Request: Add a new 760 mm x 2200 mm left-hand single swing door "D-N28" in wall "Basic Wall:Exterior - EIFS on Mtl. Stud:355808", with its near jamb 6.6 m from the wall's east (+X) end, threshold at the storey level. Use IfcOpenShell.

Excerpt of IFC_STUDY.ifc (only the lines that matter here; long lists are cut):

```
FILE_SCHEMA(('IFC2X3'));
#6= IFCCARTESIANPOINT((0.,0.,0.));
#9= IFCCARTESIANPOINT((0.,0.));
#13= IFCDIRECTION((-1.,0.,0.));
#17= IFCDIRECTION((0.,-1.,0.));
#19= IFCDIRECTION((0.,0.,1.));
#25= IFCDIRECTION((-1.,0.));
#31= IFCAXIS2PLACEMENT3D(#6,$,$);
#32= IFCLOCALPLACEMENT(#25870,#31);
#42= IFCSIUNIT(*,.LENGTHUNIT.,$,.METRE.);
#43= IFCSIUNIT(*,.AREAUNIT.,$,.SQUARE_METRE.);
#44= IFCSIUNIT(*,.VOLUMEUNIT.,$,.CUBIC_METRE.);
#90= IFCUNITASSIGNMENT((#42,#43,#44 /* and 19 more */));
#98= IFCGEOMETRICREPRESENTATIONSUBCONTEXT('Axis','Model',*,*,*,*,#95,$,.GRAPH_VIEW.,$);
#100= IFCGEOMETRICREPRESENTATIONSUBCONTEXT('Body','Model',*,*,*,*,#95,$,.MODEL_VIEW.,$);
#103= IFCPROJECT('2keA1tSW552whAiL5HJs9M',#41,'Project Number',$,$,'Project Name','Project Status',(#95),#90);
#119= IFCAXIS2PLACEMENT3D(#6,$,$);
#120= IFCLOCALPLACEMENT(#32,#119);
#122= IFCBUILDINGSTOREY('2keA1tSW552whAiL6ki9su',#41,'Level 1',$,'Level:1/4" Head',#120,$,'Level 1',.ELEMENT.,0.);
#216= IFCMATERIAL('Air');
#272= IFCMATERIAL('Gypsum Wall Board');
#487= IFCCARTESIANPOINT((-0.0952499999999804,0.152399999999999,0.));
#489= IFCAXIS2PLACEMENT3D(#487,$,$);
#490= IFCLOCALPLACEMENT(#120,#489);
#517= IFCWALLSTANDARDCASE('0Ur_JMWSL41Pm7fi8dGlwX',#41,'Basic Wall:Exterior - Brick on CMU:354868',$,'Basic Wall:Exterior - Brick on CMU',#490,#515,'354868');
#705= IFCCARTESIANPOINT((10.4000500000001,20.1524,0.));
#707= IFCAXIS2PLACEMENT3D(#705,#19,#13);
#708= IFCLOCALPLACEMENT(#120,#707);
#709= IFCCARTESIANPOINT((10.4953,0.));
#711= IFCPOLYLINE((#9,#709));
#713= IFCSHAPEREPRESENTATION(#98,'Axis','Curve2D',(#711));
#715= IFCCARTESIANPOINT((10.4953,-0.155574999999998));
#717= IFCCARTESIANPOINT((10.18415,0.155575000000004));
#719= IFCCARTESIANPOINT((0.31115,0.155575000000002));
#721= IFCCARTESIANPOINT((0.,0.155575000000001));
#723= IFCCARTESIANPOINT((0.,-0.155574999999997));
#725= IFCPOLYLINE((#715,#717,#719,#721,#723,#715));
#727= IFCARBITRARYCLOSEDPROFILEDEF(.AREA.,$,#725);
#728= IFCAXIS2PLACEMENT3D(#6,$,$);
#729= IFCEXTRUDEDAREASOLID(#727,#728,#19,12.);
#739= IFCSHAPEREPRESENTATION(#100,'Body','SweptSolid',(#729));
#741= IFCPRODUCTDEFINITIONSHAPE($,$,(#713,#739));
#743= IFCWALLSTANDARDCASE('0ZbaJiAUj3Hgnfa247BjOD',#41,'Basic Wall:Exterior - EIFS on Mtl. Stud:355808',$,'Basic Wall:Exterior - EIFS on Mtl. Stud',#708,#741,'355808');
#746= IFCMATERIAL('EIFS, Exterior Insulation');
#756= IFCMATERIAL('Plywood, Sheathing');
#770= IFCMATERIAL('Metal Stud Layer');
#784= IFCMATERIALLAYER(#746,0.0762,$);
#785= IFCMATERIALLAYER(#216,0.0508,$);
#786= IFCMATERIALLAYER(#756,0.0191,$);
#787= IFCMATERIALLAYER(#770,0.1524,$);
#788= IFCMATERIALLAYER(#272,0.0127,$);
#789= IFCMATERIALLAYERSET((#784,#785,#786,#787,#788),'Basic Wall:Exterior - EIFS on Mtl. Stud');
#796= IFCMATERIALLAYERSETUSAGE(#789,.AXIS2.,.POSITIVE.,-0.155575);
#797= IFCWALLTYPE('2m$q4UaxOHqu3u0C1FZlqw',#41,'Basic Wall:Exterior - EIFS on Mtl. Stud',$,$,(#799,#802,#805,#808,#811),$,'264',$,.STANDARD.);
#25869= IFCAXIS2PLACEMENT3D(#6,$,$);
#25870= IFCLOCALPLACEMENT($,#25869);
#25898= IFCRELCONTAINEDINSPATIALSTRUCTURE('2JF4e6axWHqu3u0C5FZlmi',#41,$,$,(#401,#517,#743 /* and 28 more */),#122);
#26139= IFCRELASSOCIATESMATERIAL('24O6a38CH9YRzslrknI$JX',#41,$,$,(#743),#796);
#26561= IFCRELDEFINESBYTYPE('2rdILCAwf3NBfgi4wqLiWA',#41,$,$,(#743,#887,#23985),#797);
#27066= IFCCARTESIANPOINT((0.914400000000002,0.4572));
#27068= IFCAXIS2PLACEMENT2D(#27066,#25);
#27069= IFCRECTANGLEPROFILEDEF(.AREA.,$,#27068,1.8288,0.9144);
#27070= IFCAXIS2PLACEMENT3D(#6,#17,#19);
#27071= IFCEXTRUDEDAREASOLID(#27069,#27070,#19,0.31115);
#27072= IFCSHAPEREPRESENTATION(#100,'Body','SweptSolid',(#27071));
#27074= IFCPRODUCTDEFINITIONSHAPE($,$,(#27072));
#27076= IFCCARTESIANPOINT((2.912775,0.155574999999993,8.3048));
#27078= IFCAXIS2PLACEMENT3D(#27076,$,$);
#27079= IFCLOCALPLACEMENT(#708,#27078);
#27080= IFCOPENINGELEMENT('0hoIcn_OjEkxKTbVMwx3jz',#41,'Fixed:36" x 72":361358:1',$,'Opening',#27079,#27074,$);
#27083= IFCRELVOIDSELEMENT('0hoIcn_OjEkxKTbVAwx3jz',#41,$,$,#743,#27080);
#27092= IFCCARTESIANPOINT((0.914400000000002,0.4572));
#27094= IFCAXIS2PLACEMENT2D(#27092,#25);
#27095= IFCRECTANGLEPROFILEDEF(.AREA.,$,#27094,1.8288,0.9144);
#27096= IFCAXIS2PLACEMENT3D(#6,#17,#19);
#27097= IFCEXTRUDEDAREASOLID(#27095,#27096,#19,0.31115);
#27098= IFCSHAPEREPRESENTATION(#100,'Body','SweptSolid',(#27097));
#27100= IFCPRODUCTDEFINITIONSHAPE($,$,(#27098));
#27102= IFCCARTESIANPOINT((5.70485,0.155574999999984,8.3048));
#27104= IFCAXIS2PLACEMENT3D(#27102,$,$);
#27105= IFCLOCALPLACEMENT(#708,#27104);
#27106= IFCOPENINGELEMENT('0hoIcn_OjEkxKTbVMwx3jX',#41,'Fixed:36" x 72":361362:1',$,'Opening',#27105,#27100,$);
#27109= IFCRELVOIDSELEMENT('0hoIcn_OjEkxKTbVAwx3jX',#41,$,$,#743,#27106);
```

```python
import numpy as np
import ifcopenshell
import ifcopenshell.api.feature
import ifcopenshell.api.geometry
import ifcopenshell.api.root
import ifcopenshell.api.spatial
import ifcopenshell.api.type
import ifcopenshell.geom
import ifcopenshell.util.element
import ifcopenshell.util.placement
import ifcopenshell.util.representation
import ifcopenshell.util.shape
import ifcopenshell.util.unit

model = ifcopenshell.open("IFC_STUDY.ifc")
unit_scale = ifcopenshell.util.unit.calculate_unit_scale(model)
settings = ifcopenshell.geom.settings()


def volume(element):
    """Net volume in cubic metres, openings subtracted."""
    shape = ifcopenshell.geom.create_shape(settings, element)
    return ifcopenshell.util.shape.get_volume(shape.geometry)


wall = model.by_id(743)
storey = ifcopenshell.util.element.get_container(wall, ifc_class="IfcBuildingStorey")
context = ifcopenshell.util.representation.get_context(model, "Model", "Body", "MODEL_VIEW")
before = volume(wall)

width, height, from_end, sill = 0.76, 2.2, 6.6, 0.0  # metres

# The wall runs along its own X axis, and the end named is its -X end.
wall_shape = ifcopenshell.geom.create_shape(settings, wall)
x, y, z = ifcopenshell.util.shape.get_vertices(wall_shape.geometry).T
start = x.min() + from_end
face, thickness = float(y.min()), float(y.max() - y.min())
wall_matrix = ifcopenshell.util.placement.get_local_placement(wall.ObjectPlacement)
level = ifcopenshell.util.placement.get_local_placement(storey.ObjectPlacement)[2, 3]


def in_wall(x, y):
    """Placement at x, y metres in the wall's axes, at sill height."""
    matrix = wall_matrix.copy()
    matrix[:, 3] = wall_matrix @ np.array([x / unit_scale, y / unit_scale, 0.0, 1.0])
    matrix[2, 3] = level + sill / unit_scale
    return matrix


# Opening: a box that overshoots both wall faces by 50 mm.
opening = ifcopenshell.api.root.create_entity(model, ifc_class="IfcOpeningElement")
box = ifcopenshell.api.geometry.add_wall_representation(
    model, context=context, length=width, height=height, thickness=thickness + 0.1
)
ifcopenshell.api.geometry.assign_representation(model, product=opening, representation=box)
ifcopenshell.api.geometry.edit_object_placement(model, product=opening, matrix=in_wall(start, face - 0.05), is_si=False)
ifcopenshell.api.feature.add_feature(model, feature=opening, element=wall)

door = ifcopenshell.api.root.create_entity(model, ifc_class="IfcDoor", name="D-N28")
door.OverallWidth, door.OverallHeight = width / unit_scale, height / unit_scale
body = ifcopenshell.api.geometry.add_door_representation(
    model,
    context=context,
    overall_width=door.OverallWidth,
    overall_height=door.OverallHeight,
    operation_type="SINGLE_SWING_LEFT",
    lining_properties={"LiningDepth": thickness / unit_scale, "ThresholdDepth": thickness / unit_scale},
)
ifcopenshell.api.geometry.assign_representation(model, product=door, representation=body)
ifcopenshell.api.spatial.assign_container(model, products=[door], relating_structure=storey)
fills = ifcopenshell.api.feature.add_filling(model, opening=opening, element=door)
fills.OwnerHistory = door.OwnerHistory  # required in IFC2X3

# IFC2X3 keeps the operation on the door style.
style = ifcopenshell.api.root.create_entity(model, ifc_class="IfcDoorStyle", name="D-N28")
style.OperationType, style.ConstructionType = "SINGLE_SWING_LEFT", "NOTDEFINED"
style.ParameterTakesPrecedence = style.Sizeable = False
ifcopenshell.api.type.assign_type(model, related_objects=[door], relating_type=style)

# The lining spans the wall, so the door starts at the wall face.
ifcopenshell.api.geometry.edit_object_placement(model, product=door, matrix=in_wall(start, face), is_si=False)

after = volume(wall)

print(f"wall volume {before:.3f} -> {after:.3f} m3")

model.write("IFC_STUDY_updated.ifc")
```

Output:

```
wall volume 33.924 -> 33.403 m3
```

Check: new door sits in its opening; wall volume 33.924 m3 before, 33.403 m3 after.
